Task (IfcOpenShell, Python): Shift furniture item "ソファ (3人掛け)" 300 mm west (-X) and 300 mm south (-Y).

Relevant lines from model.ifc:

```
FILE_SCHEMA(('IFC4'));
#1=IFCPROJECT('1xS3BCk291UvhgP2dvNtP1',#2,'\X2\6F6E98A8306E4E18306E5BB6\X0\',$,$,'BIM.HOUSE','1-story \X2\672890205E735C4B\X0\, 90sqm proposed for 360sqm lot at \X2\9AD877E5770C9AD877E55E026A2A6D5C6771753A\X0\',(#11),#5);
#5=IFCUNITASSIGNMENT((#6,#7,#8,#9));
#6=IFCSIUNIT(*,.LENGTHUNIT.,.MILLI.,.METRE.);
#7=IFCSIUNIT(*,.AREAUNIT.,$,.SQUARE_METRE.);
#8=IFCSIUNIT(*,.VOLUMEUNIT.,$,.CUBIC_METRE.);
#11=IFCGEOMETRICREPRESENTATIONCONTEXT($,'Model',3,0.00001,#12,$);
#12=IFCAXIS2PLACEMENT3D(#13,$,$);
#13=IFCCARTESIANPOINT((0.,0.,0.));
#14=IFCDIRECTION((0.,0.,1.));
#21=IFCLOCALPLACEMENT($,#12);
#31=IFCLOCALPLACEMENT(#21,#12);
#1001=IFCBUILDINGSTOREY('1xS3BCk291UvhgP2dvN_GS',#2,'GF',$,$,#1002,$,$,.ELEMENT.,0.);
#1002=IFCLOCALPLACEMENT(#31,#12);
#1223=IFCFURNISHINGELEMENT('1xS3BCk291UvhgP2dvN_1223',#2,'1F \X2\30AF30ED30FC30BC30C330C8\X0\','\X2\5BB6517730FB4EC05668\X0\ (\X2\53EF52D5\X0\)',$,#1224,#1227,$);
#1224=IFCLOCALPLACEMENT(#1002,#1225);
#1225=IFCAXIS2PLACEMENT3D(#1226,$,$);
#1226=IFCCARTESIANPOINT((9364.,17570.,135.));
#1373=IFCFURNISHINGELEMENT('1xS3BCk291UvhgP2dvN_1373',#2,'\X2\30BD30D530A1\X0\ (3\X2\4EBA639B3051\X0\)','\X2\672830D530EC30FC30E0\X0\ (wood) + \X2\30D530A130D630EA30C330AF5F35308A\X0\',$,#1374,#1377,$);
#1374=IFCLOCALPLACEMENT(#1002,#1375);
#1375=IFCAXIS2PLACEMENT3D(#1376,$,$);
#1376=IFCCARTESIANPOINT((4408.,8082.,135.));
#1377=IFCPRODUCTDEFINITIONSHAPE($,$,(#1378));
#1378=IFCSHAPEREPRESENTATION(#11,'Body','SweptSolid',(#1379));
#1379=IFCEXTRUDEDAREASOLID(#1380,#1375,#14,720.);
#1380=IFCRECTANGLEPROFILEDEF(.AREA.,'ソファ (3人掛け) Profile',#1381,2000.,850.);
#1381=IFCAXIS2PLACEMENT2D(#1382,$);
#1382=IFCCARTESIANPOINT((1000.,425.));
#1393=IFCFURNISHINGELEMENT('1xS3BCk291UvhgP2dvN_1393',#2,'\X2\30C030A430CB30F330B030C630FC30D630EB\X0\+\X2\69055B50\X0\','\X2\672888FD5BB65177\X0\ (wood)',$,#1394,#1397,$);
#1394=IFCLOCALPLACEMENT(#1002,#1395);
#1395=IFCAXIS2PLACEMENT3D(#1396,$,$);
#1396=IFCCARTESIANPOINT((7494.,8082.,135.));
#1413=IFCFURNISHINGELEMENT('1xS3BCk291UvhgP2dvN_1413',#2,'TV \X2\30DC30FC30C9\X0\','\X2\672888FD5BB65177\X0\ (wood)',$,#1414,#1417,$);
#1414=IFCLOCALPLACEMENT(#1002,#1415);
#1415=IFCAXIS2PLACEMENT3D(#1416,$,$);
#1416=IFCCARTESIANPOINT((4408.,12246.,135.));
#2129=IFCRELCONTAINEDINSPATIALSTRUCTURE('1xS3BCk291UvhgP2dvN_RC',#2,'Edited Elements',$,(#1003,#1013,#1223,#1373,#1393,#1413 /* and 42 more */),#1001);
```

```python
import ifcopenshell
import ifcopenshell.api.geometry
import ifcopenshell.util.placement
import ifcopenshell.util.unit

model = ifcopenshell.open("model.ifc")
unit_scale = ifcopenshell.util.unit.calculate_unit_scale(model)

item = model.by_guid("1xS3BCk291UvhgP2dvN_1373")
matrix = ifcopenshell.util.placement.get_local_placement(item.ObjectPlacement)
matrix[0, 3] -= 0.3 / unit_scale
matrix[1, 3] -= 0.3 / unit_scale
ifcopenshell.api.geometry.edit_object_placement(model, product=item, matrix=matrix, is_si=False)

print(ifcopenshell.util.placement.get_local_placement(item.ObjectPlacement).round(3) + 0.0)

model.write("model-out.ifc")
```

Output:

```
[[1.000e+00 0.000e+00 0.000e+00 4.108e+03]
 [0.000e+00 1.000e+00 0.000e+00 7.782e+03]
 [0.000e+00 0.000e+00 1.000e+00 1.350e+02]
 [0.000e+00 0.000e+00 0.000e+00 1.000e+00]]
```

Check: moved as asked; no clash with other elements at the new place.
